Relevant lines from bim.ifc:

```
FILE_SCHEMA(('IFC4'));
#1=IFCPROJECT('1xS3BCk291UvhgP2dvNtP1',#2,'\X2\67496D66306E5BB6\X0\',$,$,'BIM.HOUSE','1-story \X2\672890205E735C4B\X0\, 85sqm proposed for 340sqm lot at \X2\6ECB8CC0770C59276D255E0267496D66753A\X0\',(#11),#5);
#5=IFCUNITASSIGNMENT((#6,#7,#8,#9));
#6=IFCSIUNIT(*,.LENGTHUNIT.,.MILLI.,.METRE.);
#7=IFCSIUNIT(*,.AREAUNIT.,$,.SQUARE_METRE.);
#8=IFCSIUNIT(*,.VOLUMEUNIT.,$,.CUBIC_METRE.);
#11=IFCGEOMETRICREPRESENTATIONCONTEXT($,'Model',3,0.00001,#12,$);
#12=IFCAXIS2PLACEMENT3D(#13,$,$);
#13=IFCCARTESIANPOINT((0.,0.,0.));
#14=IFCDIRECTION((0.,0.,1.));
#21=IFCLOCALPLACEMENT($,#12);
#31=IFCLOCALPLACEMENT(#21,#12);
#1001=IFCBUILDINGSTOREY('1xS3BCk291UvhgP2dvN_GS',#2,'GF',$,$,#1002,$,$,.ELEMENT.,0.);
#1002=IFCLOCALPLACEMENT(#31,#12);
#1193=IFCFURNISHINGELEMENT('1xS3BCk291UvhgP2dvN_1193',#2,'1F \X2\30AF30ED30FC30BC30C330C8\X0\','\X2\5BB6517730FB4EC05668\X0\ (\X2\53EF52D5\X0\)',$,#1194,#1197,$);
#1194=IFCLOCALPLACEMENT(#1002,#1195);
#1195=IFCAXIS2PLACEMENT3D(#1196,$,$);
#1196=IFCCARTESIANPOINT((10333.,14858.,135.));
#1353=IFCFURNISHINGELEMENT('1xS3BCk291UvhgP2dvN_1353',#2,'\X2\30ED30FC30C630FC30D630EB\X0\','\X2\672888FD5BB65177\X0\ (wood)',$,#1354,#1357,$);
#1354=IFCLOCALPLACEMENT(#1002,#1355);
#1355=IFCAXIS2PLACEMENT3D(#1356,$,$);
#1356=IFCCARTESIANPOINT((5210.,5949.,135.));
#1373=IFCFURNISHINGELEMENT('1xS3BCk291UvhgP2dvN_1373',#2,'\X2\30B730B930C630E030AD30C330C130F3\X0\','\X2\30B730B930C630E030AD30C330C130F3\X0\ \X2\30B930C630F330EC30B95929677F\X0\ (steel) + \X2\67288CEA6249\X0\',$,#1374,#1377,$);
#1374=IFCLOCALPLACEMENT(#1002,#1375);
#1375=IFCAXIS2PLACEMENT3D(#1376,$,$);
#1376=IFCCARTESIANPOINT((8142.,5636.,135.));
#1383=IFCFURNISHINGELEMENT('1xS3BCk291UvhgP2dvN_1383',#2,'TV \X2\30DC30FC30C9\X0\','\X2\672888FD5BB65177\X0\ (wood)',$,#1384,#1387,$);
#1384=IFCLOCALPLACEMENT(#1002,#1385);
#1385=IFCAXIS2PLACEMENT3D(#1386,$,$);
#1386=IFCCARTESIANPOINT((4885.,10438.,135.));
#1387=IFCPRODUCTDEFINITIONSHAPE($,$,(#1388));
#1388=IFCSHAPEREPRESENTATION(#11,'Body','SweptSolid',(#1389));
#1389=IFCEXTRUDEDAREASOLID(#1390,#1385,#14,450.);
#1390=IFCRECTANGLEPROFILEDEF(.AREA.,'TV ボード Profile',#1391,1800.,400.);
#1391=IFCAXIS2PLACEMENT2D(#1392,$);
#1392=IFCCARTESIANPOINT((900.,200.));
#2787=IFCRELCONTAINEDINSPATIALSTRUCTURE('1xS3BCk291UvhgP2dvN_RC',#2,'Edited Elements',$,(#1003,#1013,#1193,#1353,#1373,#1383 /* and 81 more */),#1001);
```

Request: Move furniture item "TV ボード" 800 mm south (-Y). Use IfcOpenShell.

```python
import ifcopenshell
import ifcopenshell.api.geometry
import ifcopenshell.util.placement

model = ifcopenshell.open("bim.ifc")

item = model.by_guid("1xS3BCk291UvhgP2dvN_1383")
matrix = ifcopenshell.util.placement.get_local_placement(item.ObjectPlacement)
matrix[1, 3] -= 800.0
ifcopenshell.api.geometry.edit_object_placement(model, product=item, matrix=matrix, is_si=False)

print(ifcopenshell.util.placement.get_local_placement(item.ObjectPlacement).round(3) + 0.0)

model.write("bim_v2.ifc")
```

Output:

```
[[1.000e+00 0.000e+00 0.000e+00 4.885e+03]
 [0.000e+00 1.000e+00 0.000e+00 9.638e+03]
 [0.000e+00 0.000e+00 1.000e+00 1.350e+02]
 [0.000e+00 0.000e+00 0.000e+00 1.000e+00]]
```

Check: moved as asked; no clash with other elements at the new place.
